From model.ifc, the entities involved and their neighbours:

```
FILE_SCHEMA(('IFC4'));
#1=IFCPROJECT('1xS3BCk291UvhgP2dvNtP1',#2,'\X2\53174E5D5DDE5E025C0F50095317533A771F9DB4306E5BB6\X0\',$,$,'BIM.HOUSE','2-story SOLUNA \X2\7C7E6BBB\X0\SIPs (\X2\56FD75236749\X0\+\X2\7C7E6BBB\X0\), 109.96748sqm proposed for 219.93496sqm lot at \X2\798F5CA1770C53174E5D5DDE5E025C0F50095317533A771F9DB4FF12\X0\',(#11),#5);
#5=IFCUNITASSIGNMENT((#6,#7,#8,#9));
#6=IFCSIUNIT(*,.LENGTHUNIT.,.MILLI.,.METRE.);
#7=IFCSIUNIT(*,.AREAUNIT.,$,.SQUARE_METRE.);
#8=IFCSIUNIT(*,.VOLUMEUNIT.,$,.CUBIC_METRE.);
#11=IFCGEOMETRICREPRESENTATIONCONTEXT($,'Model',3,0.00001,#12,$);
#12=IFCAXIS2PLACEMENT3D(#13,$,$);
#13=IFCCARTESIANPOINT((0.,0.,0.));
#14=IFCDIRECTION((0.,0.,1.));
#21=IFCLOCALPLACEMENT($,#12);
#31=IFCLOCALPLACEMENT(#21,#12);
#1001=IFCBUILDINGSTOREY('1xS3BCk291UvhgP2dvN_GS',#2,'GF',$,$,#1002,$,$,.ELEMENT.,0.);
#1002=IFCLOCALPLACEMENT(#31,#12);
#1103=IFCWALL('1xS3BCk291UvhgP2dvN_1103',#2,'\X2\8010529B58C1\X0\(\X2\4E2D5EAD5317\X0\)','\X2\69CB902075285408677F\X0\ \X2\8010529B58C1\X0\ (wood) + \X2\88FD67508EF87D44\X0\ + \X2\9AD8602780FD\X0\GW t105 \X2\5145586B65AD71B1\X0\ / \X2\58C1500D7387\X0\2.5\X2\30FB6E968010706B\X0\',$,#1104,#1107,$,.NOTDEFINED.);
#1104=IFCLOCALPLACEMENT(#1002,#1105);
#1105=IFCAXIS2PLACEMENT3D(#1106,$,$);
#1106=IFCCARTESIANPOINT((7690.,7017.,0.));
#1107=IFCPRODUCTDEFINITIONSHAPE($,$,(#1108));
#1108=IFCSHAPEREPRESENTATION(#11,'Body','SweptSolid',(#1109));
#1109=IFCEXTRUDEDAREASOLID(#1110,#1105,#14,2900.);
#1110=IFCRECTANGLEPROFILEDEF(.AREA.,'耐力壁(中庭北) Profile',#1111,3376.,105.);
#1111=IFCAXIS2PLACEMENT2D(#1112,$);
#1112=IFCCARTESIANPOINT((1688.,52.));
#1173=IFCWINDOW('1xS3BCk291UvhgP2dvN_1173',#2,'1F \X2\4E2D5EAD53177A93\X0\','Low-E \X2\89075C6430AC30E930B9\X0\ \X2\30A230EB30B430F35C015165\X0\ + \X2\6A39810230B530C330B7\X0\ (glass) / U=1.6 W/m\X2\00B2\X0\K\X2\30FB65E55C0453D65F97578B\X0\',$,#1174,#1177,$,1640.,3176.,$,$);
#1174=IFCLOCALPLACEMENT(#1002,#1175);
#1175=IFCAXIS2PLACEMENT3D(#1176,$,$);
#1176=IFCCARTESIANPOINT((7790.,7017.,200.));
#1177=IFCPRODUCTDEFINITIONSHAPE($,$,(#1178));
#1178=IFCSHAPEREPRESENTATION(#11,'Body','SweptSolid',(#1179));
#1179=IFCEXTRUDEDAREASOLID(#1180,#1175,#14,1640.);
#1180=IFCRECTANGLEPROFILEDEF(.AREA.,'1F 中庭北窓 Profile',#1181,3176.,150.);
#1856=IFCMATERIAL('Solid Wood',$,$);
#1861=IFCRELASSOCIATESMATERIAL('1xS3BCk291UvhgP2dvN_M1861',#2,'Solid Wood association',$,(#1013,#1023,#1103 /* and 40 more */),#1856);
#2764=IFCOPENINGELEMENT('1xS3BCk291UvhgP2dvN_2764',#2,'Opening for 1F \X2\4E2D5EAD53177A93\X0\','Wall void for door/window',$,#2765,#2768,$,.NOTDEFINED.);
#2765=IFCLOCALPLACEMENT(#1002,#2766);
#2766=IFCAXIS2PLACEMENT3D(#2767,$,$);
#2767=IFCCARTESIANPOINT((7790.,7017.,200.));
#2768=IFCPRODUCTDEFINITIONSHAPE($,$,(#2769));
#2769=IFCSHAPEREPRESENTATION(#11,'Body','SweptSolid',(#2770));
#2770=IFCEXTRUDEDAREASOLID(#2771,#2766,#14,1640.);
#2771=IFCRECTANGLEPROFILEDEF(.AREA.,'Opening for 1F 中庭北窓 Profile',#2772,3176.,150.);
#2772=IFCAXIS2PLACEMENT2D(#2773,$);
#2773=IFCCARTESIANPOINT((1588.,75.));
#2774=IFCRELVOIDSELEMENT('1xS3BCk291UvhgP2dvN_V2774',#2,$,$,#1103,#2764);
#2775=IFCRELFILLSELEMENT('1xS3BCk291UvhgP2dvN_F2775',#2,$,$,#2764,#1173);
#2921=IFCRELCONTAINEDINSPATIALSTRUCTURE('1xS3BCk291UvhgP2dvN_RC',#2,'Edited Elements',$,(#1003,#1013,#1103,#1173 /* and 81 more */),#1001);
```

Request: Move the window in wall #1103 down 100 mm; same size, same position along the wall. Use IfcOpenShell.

```python
import numpy as np
import ifcopenshell
import ifcopenshell.api.geometry
import ifcopenshell.util.placement
import ifcopenshell.util.unit

model = ifcopenshell.open("model.ifc")
unit_scale = ifcopenshell.util.unit.calculate_unit_scale(model)

window = model.by_id(1173)
opening = window.FillsVoids[0].RelatingOpeningElement
dz = -0.1 / unit_scale

shift = np.array([0.0, 0.0, dz])
# The window is not placed relative to its opening, so move both.
for product in (opening, window):
    matrix = ifcopenshell.util.placement.get_local_placement(product.ObjectPlacement)
    matrix[:3, 3] += shift
    ifcopenshell.api.geometry.edit_object_placement(model, product=product, matrix=matrix, is_si=False)

print(f"moved by {dz * unit_scale:+.3f} m")

model.write("model_rev.ifc")
```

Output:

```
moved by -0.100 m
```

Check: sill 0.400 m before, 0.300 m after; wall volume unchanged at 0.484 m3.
